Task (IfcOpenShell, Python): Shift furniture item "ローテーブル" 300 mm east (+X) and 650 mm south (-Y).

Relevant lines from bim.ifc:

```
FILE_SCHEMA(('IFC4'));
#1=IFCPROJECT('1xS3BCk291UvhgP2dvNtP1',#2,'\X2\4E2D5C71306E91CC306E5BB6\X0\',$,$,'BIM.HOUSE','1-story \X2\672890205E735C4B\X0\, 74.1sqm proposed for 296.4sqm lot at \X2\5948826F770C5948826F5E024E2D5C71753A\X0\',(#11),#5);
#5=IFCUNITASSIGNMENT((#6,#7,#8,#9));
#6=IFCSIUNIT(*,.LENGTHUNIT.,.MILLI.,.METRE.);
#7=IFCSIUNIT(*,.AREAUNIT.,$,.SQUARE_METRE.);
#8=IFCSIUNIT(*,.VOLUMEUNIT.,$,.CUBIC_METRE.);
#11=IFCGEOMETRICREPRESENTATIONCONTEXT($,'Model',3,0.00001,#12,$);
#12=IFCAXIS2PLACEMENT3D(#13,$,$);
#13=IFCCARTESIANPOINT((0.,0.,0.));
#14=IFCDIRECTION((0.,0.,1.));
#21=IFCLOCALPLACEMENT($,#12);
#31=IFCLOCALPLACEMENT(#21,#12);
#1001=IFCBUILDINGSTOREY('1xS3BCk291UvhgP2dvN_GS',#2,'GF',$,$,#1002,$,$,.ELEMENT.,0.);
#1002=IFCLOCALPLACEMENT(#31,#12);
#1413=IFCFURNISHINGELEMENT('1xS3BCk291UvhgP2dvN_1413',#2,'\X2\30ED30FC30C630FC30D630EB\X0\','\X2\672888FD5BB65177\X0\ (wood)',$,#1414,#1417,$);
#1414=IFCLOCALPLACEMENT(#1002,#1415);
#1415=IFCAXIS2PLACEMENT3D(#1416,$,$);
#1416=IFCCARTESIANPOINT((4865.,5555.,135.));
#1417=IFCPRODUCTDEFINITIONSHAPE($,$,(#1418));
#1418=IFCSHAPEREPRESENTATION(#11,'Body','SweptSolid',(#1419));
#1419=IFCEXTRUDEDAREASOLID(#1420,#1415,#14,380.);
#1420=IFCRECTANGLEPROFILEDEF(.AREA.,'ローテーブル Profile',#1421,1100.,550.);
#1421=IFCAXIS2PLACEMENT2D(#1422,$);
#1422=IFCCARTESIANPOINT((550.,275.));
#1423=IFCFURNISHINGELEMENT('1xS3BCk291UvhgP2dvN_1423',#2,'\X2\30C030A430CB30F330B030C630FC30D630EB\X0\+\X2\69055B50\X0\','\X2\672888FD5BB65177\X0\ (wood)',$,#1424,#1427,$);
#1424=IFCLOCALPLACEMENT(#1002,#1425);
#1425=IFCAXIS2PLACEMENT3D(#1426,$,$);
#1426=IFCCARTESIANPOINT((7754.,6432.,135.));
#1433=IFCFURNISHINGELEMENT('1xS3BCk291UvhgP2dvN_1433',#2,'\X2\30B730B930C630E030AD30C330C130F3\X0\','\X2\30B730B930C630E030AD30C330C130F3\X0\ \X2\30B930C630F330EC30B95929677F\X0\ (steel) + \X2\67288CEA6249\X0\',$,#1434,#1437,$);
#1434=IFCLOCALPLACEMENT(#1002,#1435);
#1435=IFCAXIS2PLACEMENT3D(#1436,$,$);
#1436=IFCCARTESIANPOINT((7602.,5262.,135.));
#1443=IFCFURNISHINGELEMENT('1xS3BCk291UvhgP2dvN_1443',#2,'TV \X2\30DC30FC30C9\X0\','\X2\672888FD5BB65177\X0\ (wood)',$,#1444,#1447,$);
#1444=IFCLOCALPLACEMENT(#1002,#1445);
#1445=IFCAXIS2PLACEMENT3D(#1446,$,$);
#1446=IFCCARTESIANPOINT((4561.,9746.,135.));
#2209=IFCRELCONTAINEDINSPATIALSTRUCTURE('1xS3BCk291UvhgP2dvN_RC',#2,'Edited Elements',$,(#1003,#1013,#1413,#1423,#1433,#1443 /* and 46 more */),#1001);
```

```python
import ifcopenshell
import ifcopenshell.api.geometry
import ifcopenshell.util.placement
import ifcopenshell.util.unit

model = ifcopenshell.open("bim.ifc")
unit_scale = ifcopenshell.util.unit.calculate_unit_scale(model)

item = model.by_id(1413)
matrix = ifcopenshell.util.placement.get_local_placement(item.ObjectPlacement)
matrix[0, 3] += 0.3 / unit_scale
matrix[1, 3] -= 0.65 / unit_scale
ifcopenshell.api.geometry.edit_object_placement(model, product=item, matrix=matrix, is_si=False)

print(ifcopenshell.util.placement.get_local_placement(item.ObjectPlacement).round(3) + 0.0)

model.write("bim_rev.ifc")
```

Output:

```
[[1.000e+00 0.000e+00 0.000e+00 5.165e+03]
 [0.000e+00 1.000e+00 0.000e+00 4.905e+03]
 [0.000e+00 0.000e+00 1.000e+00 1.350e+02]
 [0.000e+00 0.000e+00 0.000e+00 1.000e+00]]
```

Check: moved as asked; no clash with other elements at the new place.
